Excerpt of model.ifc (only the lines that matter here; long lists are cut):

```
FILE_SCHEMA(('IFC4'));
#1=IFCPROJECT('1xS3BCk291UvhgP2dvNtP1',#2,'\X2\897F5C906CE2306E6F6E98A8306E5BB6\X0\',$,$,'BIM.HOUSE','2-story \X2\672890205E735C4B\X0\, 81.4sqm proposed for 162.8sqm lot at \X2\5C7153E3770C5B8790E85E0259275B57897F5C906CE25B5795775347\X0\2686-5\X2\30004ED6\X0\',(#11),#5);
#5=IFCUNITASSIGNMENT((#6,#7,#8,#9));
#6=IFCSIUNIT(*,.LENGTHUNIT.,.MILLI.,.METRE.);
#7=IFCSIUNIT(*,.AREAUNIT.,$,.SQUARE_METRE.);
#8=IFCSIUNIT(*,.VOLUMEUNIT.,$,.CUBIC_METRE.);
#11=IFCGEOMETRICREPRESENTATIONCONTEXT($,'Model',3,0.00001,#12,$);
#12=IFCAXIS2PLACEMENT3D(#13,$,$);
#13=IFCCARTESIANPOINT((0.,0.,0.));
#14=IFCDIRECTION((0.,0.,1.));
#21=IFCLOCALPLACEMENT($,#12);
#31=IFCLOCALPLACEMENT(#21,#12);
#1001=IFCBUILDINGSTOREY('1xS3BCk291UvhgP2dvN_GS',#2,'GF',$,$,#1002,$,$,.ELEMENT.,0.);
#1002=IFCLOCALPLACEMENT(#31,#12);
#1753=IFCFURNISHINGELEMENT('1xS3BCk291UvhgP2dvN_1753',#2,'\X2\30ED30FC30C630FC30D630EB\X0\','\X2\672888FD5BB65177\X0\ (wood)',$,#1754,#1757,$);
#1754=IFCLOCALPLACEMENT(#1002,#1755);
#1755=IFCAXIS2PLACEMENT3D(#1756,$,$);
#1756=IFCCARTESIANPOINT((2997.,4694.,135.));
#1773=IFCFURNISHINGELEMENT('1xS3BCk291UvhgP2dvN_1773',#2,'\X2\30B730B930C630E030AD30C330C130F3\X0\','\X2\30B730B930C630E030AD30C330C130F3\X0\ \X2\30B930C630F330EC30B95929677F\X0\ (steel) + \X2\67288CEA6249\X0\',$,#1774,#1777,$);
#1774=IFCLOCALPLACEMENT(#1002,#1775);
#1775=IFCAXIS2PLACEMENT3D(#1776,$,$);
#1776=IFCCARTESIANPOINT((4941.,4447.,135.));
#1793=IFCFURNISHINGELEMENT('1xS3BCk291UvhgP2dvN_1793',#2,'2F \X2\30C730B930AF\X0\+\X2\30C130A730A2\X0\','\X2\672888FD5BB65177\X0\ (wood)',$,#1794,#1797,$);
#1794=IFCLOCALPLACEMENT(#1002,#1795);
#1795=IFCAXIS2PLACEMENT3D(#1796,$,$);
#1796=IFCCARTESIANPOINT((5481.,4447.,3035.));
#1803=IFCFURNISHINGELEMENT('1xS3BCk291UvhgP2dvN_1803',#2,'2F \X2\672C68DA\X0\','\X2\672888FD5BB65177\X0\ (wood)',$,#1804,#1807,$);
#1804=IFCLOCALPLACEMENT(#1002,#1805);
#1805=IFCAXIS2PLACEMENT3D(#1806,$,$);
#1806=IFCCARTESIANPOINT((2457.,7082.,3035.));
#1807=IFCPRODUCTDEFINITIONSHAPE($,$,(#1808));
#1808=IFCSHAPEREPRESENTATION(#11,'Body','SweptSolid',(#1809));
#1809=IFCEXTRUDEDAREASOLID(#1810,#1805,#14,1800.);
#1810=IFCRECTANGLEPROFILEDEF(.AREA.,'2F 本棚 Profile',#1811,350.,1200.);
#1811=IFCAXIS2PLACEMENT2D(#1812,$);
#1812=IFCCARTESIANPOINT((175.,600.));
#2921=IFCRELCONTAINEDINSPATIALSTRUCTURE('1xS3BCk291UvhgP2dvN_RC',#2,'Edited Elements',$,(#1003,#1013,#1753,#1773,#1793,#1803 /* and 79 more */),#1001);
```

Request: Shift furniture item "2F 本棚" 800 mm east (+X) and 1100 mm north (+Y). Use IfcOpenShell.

```python
import ifcopenshell
import ifcopenshell.api.geometry
import ifcopenshell.util.placement
import ifcopenshell.util.unit

model = ifcopenshell.open("model.ifc")
unit_scale = ifcopenshell.util.unit.calculate_unit_scale(model)

item = model.by_guid("1xS3BCk291UvhgP2dvN_1803")
matrix = ifcopenshell.util.placement.get_local_placement(item.ObjectPlacement)
matrix[0, 3] += 0.8 / unit_scale
matrix[1, 3] += 1.1 / unit_scale
ifcopenshell.api.geometry.edit_object_placement(model, product=item, matrix=matrix, is_si=False)

print(ifcopenshell.util.placement.get_local_placement(item.ObjectPlacement).round(3) + 0.0)

model.write("model_rev.ifc")
```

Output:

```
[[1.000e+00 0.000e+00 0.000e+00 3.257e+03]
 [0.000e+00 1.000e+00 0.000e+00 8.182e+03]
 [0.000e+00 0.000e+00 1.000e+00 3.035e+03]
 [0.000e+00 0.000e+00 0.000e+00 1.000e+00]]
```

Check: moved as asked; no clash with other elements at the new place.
